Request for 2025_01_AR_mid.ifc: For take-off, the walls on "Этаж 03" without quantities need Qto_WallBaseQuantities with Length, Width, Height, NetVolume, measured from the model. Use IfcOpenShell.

First a look at what the model holds.

```python
import ifcopenshell
import ifcopenshell.util.element
import ifcopenshell.util.unit

model = ifcopenshell.open("2025_01_AR_mid.ifc")
print(model.schema)
for unit_type in ("LENGTHUNIT", "AREAUNIT", "VOLUMEUNIT"):
    print(unit_type, ifcopenshell.util.unit.calculate_unit_scale(model, unit_type))
storey = next(s for s in model.by_type("IfcBuildingStorey") if s.Name == "Этаж 03")
walls = [e for e in ifcopenshell.util.element.get_decomposition(storey) if e.is_a("IfcWall")]
for e in sorted(walls, key=lambda e: e.id()):
    print(e.id(), e.is_a(), e.Name, list(ifcopenshell.util.element.get_psets(e, qtos_only=True)), sep=" | ")
```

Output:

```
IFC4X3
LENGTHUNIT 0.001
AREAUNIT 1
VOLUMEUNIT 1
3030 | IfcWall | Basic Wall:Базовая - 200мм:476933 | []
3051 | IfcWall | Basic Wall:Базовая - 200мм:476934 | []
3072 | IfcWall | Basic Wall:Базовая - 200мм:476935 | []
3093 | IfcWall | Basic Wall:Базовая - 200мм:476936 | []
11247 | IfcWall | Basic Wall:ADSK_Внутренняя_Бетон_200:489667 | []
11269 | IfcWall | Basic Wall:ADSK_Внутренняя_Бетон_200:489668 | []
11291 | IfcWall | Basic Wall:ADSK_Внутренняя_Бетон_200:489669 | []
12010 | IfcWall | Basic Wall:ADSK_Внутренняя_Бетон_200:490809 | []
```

```python
import ifcopenshell
import ifcopenshell.api.pset
import ifcopenshell.geom
import ifcopenshell.util.element
import ifcopenshell.util.shape
import ifcopenshell.util.unit

model = ifcopenshell.open("2025_01_AR_mid.ifc")
unit_scale = ifcopenshell.util.unit.calculate_unit_scale(model)
volume_scale = ifcopenshell.util.unit.calculate_unit_scale(model, "VOLUMEUNIT")
settings = ifcopenshell.geom.settings()

storey = next(s for s in model.by_type("IfcBuildingStorey") if s.Name == "Этаж 03")
walls = [e for e in ifcopenshell.util.element.get_decomposition(storey) if e.is_a("IfcWall")]

for e in sorted(walls, key=lambda e: e.id()):
    if ifcopenshell.util.element.get_psets(e, qtos_only=True, should_inherit=False):
        continue
    # Geometry comes back in metres, in the element's own axes.
    shape = ifcopenshell.geom.create_shape(settings, e)
    values = {
        "Length": ifcopenshell.util.shape.get_x(shape.geometry) / unit_scale,
        "Width": ifcopenshell.util.shape.get_y(shape.geometry) / unit_scale,
        "Height": ifcopenshell.util.shape.get_z(shape.geometry) / unit_scale,
        "NetVolume": ifcopenshell.util.shape.get_volume(shape.geometry) / volume_scale,
    }
    qto = ifcopenshell.api.pset.add_qto(model, product=e, name="Qto_WallBaseQuantities")
    ifcopenshell.api.pset.edit_qto(model, qto=qto, properties=values)
    print(e.id(), {k: round(v, 3) for k, v in values.items()})

model.write("2025_01_AR_mid_rev.ifc")
```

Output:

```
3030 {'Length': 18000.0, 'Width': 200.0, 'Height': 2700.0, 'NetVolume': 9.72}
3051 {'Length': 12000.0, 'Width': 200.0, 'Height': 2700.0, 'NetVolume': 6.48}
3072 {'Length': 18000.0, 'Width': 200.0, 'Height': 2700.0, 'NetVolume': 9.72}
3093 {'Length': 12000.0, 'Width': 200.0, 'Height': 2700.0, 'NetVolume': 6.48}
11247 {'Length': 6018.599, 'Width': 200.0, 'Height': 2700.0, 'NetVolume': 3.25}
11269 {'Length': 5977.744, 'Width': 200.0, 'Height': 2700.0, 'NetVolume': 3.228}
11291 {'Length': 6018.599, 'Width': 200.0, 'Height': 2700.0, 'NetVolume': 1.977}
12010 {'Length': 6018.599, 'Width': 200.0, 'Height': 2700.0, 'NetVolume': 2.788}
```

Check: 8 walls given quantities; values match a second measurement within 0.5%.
